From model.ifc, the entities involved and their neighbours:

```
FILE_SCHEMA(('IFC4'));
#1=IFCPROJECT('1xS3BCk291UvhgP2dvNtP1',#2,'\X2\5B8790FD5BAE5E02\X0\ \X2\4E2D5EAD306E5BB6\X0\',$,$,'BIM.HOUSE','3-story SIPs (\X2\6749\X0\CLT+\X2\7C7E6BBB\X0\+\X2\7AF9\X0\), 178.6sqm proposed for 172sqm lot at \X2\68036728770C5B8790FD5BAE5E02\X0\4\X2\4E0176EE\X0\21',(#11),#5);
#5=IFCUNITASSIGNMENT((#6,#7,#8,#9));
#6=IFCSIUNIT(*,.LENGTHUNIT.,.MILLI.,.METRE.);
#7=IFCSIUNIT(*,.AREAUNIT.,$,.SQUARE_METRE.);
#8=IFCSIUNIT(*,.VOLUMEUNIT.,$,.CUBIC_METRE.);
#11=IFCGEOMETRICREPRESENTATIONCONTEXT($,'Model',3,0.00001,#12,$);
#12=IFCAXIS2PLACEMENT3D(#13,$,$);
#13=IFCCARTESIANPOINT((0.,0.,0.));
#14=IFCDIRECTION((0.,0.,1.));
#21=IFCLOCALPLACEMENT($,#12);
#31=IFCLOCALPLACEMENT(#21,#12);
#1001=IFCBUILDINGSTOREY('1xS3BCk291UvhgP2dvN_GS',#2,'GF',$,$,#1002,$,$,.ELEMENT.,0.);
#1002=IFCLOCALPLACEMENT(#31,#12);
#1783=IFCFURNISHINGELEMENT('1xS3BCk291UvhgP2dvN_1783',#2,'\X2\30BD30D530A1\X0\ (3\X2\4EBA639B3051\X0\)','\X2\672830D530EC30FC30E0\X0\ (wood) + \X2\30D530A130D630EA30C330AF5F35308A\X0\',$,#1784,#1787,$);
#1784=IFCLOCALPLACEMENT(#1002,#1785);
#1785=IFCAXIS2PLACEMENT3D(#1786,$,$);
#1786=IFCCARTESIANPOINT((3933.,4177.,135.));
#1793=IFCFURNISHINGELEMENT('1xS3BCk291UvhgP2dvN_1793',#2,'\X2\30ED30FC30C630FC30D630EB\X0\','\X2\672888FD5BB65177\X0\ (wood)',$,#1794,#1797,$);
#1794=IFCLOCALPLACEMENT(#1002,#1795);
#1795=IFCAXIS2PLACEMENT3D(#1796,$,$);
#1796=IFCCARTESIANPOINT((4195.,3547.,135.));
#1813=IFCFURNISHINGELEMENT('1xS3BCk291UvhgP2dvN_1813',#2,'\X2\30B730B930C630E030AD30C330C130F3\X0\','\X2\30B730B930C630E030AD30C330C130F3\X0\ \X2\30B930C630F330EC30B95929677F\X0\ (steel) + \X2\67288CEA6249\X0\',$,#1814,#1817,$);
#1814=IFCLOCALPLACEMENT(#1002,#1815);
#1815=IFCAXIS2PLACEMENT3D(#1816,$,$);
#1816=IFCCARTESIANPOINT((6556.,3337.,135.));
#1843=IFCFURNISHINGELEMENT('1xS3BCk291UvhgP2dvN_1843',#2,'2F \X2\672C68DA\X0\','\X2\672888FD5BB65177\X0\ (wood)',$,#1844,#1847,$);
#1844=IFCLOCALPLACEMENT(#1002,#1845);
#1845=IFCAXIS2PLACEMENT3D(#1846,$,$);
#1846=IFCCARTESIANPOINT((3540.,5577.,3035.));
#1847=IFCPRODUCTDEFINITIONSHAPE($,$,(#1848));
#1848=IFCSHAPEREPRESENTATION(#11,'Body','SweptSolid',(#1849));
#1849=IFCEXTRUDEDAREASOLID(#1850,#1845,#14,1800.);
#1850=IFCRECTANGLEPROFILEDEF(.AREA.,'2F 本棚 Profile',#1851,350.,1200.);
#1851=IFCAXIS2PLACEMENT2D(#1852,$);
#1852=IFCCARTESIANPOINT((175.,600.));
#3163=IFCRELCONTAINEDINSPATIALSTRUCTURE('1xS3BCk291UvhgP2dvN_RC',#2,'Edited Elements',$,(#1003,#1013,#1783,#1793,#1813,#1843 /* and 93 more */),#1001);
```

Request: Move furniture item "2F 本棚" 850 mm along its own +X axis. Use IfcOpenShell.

```python
import ifcopenshell
import ifcopenshell.api.geometry
import ifcopenshell.util.placement
import ifcopenshell.util.unit

model = ifcopenshell.open("model.ifc")
unit_scale = ifcopenshell.util.unit.calculate_unit_scale(model)

item = model.by_guid("1xS3BCk291UvhgP2dvN_1843")
matrix = ifcopenshell.util.placement.get_local_placement(item.ObjectPlacement)
matrix[:3, 3] += matrix[:3, 0] * 0.85 / unit_scale
ifcopenshell.api.geometry.edit_object_placement(model, product=item, matrix=matrix, is_si=False)

print(ifcopenshell.util.placement.get_local_placement(item.ObjectPlacement).round(3) + 0.0)

model.write("model_edited.ifc")
```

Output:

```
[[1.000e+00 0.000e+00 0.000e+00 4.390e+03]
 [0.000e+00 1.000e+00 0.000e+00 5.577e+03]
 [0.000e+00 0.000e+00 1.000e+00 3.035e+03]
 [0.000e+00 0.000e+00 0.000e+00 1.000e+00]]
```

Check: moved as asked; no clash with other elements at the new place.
